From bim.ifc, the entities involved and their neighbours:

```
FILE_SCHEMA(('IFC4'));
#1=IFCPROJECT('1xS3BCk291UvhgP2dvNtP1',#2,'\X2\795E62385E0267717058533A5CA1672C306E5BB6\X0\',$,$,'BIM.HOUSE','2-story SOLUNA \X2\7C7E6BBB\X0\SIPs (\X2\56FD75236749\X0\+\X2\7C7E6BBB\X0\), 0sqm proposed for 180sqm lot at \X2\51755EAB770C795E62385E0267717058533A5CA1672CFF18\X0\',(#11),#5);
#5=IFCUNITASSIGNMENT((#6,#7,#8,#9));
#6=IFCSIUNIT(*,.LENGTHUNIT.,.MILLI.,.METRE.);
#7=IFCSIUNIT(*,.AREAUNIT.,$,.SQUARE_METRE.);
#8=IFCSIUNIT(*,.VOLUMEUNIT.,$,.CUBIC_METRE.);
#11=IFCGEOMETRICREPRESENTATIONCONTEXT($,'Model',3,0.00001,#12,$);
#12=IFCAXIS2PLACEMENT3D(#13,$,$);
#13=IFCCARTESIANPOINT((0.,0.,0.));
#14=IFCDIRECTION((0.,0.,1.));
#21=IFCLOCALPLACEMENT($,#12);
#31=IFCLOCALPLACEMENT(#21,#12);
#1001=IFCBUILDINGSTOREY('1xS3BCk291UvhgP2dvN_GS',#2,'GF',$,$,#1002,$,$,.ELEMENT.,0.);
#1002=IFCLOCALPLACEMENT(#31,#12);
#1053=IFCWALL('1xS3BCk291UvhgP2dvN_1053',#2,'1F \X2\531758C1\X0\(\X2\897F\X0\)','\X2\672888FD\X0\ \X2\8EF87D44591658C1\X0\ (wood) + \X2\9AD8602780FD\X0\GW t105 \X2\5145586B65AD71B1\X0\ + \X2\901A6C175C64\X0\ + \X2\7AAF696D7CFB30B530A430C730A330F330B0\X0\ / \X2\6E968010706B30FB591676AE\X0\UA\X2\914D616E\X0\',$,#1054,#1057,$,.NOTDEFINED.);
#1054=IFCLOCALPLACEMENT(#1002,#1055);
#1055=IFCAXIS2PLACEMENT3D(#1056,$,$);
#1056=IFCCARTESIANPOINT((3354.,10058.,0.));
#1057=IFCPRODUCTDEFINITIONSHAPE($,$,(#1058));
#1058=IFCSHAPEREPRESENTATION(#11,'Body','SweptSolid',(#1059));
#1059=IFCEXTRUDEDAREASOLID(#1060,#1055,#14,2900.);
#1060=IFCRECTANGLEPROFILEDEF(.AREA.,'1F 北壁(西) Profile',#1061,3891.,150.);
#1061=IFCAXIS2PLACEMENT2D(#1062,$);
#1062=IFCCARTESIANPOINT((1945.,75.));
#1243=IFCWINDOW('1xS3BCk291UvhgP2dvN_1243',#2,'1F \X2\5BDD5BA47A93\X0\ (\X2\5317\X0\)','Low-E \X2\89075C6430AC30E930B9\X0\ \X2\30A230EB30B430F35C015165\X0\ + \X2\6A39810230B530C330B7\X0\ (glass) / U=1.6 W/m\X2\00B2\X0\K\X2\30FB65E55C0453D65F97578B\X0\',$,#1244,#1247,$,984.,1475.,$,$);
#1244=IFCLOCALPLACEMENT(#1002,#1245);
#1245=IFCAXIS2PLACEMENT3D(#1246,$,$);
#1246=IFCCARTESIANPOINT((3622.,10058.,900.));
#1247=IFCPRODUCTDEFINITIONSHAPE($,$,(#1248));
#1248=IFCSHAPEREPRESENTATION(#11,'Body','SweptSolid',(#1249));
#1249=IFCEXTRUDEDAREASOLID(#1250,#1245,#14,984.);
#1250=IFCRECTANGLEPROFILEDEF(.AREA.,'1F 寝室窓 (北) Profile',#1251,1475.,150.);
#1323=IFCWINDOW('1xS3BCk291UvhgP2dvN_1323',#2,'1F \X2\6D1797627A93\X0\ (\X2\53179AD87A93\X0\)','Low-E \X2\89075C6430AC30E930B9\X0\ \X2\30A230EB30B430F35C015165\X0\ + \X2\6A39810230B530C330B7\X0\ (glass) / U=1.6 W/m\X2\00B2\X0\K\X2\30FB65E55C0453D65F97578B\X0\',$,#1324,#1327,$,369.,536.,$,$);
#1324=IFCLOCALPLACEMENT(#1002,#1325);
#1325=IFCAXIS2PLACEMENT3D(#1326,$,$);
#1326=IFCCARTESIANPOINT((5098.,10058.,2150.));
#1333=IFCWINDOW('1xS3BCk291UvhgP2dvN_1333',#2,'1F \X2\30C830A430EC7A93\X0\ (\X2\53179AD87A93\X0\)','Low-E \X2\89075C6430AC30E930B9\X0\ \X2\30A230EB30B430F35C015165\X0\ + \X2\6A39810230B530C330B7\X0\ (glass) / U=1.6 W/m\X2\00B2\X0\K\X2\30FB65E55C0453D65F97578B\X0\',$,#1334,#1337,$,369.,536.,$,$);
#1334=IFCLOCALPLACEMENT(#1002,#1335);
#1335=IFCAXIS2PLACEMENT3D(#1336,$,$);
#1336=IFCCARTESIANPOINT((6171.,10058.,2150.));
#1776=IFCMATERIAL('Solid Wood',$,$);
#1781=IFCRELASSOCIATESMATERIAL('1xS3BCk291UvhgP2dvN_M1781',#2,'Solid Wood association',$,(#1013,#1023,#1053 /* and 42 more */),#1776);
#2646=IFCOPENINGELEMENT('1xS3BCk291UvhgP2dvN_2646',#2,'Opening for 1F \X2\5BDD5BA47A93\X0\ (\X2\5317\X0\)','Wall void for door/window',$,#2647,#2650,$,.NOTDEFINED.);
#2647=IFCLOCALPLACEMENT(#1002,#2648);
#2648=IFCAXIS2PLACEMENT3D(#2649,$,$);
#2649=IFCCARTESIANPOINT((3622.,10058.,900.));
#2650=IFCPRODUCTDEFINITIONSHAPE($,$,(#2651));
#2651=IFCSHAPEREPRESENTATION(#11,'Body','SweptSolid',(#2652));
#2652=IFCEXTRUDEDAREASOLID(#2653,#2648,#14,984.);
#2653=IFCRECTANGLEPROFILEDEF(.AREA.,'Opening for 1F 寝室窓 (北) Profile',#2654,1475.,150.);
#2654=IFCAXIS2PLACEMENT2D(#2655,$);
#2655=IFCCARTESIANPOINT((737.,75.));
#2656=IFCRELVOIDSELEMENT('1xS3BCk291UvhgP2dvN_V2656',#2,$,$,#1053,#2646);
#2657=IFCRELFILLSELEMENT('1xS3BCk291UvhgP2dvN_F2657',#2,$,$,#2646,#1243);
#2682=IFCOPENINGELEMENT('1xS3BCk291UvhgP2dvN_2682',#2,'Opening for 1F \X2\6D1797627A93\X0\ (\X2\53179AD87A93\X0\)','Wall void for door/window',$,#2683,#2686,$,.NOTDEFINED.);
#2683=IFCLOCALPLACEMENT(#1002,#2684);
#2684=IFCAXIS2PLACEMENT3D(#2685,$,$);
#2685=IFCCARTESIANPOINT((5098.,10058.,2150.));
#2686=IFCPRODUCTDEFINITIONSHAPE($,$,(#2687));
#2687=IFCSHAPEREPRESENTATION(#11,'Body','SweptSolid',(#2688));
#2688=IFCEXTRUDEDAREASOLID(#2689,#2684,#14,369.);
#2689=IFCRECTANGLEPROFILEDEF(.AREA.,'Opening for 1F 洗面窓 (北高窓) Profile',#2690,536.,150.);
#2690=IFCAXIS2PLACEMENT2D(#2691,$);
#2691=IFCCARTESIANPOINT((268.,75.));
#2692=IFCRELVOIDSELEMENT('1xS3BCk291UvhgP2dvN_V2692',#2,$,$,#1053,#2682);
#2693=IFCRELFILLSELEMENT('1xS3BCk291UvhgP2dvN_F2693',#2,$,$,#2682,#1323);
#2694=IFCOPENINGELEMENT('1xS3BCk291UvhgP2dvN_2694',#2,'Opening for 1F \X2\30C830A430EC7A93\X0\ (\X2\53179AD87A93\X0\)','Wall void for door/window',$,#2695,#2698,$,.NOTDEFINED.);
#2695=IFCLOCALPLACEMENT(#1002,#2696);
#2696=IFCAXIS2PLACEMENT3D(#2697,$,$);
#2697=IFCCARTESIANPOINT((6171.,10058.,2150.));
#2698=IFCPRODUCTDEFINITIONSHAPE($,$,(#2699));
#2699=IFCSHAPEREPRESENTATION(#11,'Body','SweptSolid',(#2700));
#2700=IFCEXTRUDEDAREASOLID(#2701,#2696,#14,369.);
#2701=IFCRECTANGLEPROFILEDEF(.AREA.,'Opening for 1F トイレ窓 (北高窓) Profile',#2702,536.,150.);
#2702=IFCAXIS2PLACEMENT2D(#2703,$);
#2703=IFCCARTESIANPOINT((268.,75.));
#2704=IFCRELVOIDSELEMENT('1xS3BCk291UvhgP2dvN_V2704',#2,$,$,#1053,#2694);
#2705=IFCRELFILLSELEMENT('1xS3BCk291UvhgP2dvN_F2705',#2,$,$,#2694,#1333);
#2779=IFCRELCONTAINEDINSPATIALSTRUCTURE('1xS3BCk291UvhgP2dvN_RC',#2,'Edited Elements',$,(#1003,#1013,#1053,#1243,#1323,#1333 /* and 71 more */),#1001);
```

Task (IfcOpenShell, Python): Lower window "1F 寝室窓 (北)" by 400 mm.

```python
import numpy as np
import ifcopenshell
import ifcopenshell.api.geometry
import ifcopenshell.util.placement
import ifcopenshell.util.unit

model = ifcopenshell.open("bim.ifc")
unit_scale = ifcopenshell.util.unit.calculate_unit_scale(model)

window = model.by_guid("1xS3BCk291UvhgP2dvN_1243")
opening = window.FillsVoids[0].RelatingOpeningElement
dz = -400.0

shift = np.array([0.0, 0.0, dz])
# The window is not placed relative to its opening, so move both.
for product in (opening, window):
    matrix = ifcopenshell.util.placement.get_local_placement(product.ObjectPlacement)
    matrix[:3, 3] += shift
    ifcopenshell.api.geometry.edit_object_placement(model, product=product, matrix=matrix, is_si=False)

print(f"moved by {dz * unit_scale:+.3f} m")

model.write("bim_updated.ifc")
```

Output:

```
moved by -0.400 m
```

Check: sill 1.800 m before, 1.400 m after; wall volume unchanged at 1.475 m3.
